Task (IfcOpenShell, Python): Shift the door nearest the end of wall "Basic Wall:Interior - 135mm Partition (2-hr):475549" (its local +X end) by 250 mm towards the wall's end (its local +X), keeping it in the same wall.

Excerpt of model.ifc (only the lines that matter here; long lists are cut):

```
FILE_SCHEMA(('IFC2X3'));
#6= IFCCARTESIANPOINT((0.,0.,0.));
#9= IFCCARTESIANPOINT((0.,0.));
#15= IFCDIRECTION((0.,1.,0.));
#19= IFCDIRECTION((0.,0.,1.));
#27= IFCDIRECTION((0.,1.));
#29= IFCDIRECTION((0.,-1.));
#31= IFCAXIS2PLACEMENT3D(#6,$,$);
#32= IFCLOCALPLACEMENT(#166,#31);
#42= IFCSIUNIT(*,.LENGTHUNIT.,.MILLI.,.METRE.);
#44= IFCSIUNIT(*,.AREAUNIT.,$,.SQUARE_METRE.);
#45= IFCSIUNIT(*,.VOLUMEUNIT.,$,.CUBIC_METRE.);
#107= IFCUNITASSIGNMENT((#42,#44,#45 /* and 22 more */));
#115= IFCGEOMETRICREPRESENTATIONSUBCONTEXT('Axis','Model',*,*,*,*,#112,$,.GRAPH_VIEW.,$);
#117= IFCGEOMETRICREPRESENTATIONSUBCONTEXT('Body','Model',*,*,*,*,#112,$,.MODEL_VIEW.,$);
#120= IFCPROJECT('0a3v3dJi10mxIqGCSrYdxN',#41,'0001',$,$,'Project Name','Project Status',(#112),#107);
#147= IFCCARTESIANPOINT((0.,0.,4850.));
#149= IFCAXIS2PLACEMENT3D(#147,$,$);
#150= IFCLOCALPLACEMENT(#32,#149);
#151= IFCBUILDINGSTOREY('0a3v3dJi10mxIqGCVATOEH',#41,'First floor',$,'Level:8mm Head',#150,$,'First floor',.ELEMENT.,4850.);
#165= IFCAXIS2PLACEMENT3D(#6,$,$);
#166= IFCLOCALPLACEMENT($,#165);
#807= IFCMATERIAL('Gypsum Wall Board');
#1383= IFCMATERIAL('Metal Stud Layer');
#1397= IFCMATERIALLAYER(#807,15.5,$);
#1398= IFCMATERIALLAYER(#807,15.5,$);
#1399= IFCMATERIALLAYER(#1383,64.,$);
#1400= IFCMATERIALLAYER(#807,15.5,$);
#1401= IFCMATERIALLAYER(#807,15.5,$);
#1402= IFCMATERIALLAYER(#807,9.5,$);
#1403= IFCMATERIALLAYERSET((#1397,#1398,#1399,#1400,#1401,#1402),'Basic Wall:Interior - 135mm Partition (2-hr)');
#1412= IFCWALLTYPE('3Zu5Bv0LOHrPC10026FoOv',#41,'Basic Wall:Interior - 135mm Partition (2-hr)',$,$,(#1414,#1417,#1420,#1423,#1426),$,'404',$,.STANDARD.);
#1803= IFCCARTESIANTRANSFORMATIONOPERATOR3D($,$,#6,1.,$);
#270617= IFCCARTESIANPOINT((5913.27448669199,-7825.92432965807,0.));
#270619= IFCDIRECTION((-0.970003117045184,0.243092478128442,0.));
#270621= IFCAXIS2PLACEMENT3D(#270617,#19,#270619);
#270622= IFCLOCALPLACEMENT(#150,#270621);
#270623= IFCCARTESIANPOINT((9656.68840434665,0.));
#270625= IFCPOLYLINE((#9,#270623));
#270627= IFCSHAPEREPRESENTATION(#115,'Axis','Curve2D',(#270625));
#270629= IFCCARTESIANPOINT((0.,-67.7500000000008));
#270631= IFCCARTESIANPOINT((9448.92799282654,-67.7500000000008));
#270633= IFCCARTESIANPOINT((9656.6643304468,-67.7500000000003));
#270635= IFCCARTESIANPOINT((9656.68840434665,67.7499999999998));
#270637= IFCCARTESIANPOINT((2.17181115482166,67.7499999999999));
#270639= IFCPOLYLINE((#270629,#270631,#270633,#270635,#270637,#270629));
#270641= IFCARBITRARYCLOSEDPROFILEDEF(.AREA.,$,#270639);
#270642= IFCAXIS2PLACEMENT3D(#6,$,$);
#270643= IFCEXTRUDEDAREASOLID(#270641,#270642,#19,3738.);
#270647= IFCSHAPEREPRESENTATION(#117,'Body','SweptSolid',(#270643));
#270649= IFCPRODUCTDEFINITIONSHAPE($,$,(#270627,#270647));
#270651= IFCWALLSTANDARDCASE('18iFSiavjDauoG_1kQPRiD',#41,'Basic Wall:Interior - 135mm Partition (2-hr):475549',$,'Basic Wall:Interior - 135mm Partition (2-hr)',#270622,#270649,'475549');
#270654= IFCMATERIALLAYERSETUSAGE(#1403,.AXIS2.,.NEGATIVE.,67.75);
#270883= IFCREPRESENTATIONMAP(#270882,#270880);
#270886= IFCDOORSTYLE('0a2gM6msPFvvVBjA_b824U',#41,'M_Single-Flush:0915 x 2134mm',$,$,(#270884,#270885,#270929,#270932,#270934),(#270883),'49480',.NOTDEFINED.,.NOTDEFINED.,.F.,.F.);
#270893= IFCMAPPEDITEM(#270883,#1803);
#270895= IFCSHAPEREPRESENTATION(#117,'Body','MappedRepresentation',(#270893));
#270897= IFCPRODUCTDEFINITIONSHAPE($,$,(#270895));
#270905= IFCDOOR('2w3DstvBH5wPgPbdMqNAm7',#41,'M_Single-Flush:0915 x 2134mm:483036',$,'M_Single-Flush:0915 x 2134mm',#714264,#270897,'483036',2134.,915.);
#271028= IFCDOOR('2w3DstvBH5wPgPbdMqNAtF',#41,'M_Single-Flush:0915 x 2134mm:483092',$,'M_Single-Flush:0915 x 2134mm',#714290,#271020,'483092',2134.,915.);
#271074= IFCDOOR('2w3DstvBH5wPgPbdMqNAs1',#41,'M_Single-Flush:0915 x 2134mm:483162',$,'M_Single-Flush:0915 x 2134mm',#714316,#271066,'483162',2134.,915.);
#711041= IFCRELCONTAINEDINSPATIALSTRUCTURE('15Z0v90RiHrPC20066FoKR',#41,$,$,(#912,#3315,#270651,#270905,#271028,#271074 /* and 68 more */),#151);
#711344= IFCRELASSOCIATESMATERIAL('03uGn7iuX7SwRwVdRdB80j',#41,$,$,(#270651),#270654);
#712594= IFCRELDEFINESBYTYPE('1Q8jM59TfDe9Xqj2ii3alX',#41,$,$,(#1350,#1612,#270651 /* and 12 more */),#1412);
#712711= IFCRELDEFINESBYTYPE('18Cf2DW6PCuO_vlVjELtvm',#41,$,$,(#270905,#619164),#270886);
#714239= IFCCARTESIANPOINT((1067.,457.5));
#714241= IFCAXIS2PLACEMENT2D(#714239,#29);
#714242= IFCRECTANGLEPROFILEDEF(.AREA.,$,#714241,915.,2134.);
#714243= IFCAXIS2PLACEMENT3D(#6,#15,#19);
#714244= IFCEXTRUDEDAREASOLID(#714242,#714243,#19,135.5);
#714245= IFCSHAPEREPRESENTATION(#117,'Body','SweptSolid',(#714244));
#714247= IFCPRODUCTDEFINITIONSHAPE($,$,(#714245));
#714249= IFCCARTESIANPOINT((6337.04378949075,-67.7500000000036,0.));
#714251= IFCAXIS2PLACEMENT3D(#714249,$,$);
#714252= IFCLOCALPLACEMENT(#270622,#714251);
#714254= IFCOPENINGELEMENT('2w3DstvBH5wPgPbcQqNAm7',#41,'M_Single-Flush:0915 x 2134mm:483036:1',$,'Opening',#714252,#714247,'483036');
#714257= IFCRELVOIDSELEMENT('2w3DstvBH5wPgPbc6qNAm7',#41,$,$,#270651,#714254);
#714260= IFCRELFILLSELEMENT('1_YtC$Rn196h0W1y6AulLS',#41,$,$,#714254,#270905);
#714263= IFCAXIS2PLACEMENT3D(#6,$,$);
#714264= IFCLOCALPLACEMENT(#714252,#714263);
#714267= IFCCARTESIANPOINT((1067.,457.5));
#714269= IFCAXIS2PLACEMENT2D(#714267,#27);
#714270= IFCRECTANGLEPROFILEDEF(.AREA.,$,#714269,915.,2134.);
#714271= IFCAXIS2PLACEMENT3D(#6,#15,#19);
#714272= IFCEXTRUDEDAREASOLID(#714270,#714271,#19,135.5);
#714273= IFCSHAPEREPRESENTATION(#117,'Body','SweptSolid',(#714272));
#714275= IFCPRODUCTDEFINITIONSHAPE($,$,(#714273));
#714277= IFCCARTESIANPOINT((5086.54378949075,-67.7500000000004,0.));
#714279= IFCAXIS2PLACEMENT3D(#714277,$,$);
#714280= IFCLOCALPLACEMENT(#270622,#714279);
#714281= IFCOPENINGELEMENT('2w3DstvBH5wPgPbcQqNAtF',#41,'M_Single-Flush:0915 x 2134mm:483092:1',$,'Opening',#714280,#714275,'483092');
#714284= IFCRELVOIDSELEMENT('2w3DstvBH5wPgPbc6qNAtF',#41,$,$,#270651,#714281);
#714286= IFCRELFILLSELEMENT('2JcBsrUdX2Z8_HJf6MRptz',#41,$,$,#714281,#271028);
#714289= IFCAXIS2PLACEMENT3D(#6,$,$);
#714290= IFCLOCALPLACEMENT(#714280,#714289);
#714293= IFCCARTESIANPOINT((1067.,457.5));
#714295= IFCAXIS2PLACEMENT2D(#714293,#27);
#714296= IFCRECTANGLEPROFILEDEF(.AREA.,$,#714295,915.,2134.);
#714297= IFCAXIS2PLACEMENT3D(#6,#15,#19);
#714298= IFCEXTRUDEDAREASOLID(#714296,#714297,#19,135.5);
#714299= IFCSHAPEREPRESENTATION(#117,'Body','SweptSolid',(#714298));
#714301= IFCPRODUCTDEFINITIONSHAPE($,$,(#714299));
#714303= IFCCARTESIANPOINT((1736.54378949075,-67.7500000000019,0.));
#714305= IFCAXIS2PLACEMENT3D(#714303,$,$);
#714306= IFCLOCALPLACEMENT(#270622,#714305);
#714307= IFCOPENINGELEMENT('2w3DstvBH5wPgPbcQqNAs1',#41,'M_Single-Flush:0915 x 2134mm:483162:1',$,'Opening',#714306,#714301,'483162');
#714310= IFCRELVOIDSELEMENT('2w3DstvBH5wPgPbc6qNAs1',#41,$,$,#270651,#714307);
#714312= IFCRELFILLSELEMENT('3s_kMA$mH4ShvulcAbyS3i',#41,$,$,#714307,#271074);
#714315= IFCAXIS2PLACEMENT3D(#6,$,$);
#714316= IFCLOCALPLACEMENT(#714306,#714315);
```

```python
import ifcopenshell
import ifcopenshell.api.geometry
import ifcopenshell.util.placement

model = ifcopenshell.open("model.ifc")

door = model.by_guid("2w3DstvBH5wPgPbdMqNAm7")
opening = door.FillsVoids[0].RelatingOpeningElement
wall = opening.VoidsElements[0].RelatingBuildingElement

wall_matrix = ifcopenshell.util.placement.get_local_placement(wall.ObjectPlacement)
shift = wall_matrix[:3, 0] * 250.0
before = ifcopenshell.util.placement.get_local_placement(door.ObjectPlacement)[:3, 3].copy()

# The door is placed relative to its opening, so it follows when the opening moves.
matrix = ifcopenshell.util.placement.get_local_placement(opening.ObjectPlacement)
matrix[:3, 3] += shift
ifcopenshell.api.geometry.edit_object_placement(
    model, product=opening, matrix=matrix, is_si=False, should_transform_children=True
)

after = ifcopenshell.util.placement.get_local_placement(door.ObjectPlacement)[:3, 3]
print("door moved by", (after - before).round(3) + 0.0)

model.write("model-out.ifc")
```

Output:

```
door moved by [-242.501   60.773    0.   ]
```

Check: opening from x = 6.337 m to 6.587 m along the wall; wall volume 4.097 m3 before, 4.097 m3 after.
